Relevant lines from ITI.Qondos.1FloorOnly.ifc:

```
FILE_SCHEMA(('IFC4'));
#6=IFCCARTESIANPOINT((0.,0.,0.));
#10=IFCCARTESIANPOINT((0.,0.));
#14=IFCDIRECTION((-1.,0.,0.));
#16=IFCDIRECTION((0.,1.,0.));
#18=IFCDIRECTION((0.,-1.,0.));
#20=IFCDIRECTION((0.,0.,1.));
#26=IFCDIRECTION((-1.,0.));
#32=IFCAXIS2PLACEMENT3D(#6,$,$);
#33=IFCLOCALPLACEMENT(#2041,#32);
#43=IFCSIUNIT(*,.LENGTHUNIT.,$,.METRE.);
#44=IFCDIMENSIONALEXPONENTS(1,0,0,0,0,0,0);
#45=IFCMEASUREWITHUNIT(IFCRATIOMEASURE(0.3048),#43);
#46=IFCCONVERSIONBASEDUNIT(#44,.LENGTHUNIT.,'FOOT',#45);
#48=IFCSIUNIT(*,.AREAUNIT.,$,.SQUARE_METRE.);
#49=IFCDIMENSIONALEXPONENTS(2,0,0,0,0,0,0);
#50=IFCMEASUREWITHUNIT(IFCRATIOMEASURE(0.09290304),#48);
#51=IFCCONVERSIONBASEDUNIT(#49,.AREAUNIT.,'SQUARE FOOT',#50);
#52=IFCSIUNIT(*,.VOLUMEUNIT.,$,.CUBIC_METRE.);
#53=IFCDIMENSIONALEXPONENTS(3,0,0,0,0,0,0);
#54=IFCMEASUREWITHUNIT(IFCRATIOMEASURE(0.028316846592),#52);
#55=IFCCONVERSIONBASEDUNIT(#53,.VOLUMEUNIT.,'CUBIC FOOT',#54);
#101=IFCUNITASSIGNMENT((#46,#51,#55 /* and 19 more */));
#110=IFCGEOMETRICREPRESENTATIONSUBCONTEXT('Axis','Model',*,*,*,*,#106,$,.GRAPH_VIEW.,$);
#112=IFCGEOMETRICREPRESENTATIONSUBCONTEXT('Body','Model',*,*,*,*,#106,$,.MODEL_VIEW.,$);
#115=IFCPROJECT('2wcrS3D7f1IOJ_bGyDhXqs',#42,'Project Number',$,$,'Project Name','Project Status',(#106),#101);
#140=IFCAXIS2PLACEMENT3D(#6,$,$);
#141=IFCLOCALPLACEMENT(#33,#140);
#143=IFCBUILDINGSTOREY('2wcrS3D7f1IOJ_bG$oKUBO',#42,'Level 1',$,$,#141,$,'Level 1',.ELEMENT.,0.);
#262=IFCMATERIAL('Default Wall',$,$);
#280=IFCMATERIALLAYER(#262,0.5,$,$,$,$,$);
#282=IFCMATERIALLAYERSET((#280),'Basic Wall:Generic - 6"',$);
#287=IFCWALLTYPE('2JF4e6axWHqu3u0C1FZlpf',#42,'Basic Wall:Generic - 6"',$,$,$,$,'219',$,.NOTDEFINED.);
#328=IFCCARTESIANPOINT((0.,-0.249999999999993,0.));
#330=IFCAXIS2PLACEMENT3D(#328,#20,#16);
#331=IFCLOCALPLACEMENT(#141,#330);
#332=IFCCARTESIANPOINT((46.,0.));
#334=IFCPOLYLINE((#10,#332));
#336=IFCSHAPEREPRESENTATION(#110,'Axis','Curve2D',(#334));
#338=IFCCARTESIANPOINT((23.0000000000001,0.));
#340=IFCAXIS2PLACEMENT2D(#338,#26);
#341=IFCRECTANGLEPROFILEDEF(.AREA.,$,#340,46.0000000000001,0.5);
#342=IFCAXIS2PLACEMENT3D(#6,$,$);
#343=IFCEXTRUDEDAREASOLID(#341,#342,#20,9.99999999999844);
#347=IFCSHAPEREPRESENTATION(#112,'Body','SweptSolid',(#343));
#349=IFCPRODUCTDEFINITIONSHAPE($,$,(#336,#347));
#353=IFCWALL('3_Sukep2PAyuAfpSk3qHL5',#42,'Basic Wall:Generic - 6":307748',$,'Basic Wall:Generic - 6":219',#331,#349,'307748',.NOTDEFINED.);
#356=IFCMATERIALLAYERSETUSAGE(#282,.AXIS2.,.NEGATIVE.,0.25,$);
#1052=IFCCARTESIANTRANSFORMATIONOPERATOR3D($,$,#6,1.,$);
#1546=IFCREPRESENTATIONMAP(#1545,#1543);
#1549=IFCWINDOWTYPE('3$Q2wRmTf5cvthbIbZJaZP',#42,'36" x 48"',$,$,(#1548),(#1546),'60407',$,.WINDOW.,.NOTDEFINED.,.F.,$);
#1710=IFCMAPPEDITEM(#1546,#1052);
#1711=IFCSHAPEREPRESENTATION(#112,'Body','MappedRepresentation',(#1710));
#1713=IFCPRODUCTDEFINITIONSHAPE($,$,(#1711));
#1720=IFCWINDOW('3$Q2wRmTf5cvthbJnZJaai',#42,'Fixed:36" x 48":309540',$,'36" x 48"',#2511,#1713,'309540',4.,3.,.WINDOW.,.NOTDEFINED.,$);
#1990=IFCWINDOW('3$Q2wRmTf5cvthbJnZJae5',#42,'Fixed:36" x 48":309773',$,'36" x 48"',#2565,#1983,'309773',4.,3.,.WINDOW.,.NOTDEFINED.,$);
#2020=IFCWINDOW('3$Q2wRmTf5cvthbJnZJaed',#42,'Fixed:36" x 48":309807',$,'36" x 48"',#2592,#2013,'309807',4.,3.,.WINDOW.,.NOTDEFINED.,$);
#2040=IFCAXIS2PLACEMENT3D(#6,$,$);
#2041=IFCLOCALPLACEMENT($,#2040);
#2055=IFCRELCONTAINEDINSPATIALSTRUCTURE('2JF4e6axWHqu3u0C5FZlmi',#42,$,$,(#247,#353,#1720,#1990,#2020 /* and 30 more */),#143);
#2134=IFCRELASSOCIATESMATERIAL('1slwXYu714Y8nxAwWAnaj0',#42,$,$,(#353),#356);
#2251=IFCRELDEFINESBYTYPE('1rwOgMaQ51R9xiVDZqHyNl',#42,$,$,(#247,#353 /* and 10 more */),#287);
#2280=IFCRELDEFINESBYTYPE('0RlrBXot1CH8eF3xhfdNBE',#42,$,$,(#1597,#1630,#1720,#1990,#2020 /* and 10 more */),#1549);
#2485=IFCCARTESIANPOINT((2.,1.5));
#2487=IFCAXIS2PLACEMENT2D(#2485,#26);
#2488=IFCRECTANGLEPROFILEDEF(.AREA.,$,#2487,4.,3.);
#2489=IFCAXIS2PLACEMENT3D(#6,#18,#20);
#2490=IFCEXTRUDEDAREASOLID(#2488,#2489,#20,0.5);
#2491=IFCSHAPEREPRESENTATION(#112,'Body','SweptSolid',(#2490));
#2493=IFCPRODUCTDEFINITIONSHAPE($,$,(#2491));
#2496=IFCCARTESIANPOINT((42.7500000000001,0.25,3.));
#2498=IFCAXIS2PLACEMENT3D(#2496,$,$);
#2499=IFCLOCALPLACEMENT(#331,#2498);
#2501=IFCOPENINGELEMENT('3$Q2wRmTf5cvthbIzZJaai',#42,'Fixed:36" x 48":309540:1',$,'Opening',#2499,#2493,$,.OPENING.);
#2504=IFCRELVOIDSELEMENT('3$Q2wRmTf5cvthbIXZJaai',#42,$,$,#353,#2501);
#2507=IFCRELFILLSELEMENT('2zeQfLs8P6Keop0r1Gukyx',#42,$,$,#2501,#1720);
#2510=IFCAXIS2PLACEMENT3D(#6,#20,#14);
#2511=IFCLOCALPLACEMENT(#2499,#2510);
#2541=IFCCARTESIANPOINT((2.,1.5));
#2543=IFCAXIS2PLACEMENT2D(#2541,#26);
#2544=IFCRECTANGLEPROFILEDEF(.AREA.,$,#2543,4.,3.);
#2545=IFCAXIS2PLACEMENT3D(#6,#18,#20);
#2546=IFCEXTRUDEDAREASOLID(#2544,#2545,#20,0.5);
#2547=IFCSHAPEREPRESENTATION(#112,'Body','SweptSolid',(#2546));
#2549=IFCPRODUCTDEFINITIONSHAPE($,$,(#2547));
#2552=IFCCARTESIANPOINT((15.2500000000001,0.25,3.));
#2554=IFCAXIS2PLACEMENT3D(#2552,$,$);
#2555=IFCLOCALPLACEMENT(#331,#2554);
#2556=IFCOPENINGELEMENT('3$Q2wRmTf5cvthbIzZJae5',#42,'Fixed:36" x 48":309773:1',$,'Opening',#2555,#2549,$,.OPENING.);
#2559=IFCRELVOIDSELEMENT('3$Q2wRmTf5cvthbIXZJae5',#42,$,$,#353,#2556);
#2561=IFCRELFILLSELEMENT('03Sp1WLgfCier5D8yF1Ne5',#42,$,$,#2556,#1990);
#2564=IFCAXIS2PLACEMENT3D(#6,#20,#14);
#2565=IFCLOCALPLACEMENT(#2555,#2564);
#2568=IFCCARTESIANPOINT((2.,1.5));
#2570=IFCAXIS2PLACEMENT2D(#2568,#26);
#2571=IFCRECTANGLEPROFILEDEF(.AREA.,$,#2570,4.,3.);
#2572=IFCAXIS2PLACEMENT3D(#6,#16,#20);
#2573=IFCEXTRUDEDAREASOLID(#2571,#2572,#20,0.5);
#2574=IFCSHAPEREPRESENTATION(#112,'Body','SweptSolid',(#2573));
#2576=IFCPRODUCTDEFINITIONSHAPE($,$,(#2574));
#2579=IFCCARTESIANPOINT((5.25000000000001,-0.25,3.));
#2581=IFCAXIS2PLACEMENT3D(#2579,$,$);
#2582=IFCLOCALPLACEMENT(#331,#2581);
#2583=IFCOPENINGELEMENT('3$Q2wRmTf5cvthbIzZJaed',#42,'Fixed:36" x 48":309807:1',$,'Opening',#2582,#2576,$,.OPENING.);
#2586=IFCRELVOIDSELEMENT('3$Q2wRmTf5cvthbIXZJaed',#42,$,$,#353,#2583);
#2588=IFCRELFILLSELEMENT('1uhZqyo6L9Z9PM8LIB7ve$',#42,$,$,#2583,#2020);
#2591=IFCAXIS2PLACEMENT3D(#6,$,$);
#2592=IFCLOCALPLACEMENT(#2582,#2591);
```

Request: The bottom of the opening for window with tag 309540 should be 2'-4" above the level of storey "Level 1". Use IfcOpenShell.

```python
import numpy as np
import ifcopenshell
import ifcopenshell.api.geometry
import ifcopenshell.geom
import ifcopenshell.util.element
import ifcopenshell.util.placement
import ifcopenshell.util.shape
import ifcopenshell.util.unit

model = ifcopenshell.open("ITI.Qondos.1FloorOnly.ifc")
unit_scale = ifcopenshell.util.unit.calculate_unit_scale(model)

window = model.by_guid("3$Q2wRmTf5cvthbJnZJaai")
opening = window.FillsVoids[0].RelatingOpeningElement
storey = ifcopenshell.util.element.get_container(window, ifc_class="IfcBuildingStorey")
level = ifcopenshell.util.placement.get_local_placement(storey.ObjectPlacement)[2, 3]

# The opening's origin need not be at the sill, so measure its lowest point.
shape = ifcopenshell.geom.create_shape(ifcopenshell.geom.settings(), opening)
bottom = ifcopenshell.util.shape.get_shape_bottom_elevation(shape, shape.geometry) / unit_scale
dz = level + 28 * 0.0254 / unit_scale - bottom

shift = np.array([0.0, 0.0, dz])
# The window is placed relative to its opening, so it follows when the opening moves.
matrix = ifcopenshell.util.placement.get_local_placement(opening.ObjectPlacement)
matrix[:3, 3] += shift
ifcopenshell.api.geometry.edit_object_placement(
    model, product=opening, matrix=matrix, is_si=False, should_transform_children=True
)

print(f"moved by {dz * unit_scale:+.3f} m")

model.write("ITI.Qondos.1FloorOnly-out.ifc")
```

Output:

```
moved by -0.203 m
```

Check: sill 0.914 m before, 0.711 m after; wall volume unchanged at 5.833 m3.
